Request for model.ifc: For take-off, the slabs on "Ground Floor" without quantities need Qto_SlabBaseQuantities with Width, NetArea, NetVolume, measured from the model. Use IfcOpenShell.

First a look at what the model holds.

```python
import ifcopenshell
import ifcopenshell.util.element
import ifcopenshell.util.unit

model = ifcopenshell.open("model.ifc")
print(model.schema)
for unit_type in ("LENGTHUNIT", "AREAUNIT", "VOLUMEUNIT"):
    print(unit_type, ifcopenshell.util.unit.calculate_unit_scale(model, unit_type))
storey = next(s for s in model.by_type("IfcBuildingStorey") if s.Name == "Ground Floor")
slabs = [e for e in ifcopenshell.util.element.get_decomposition(storey) if e.is_a("IfcSlab")]
for e in sorted(slabs, key=lambda e: e.id()):
    print(e.id(), e.is_a(), e.Name, list(ifcopenshell.util.element.get_psets(e, qtos_only=True)), sep=" | ")
```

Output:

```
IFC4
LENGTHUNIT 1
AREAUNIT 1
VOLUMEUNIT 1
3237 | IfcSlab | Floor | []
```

```python
import ifcopenshell
import ifcopenshell.api.pset
import ifcopenshell.geom
import ifcopenshell.util.element
import ifcopenshell.util.shape
import ifcopenshell.util.unit

model = ifcopenshell.open("model.ifc")
unit_scale = ifcopenshell.util.unit.calculate_unit_scale(model)
area_scale = ifcopenshell.util.unit.calculate_unit_scale(model, "AREAUNIT")
volume_scale = ifcopenshell.util.unit.calculate_unit_scale(model, "VOLUMEUNIT")
settings = ifcopenshell.geom.settings()

storey = next(s for s in model.by_type("IfcBuildingStorey") if s.Name == "Ground Floor")
slabs = [e for e in ifcopenshell.util.element.get_decomposition(storey) if e.is_a("IfcSlab")]

for e in sorted(slabs, key=lambda e: e.id()):
    if ifcopenshell.util.element.get_psets(e, qtos_only=True, should_inherit=False):
        continue
    # Geometry comes back in metres, in the element's own axes.
    shape = ifcopenshell.geom.create_shape(settings, e)
    values = {
        "Width": ifcopenshell.util.shape.get_z(shape.geometry) / unit_scale,
        "NetArea": ifcopenshell.util.shape.get_footprint_area(shape.geometry) / area_scale,
        "NetVolume": ifcopenshell.util.shape.get_volume(shape.geometry) / volume_scale,
    }
    qto = ifcopenshell.api.pset.add_qto(model, product=e, name="Qto_SlabBaseQuantities")
    ifcopenshell.api.pset.edit_qto(model, qto=qto, properties=values)
    print(e.id(), {k: round(v, 3) for k, v in values.items()})

model.write("model_rev.ifc")
```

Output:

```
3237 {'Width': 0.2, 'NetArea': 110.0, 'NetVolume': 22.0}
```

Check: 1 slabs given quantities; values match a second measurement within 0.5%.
